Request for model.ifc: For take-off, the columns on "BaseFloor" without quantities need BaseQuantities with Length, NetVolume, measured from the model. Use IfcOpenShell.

First a look at what the model holds.

```python
import ifcopenshell
import ifcopenshell.util.element
import ifcopenshell.util.unit

model = ifcopenshell.open("model.ifc")
print(model.schema)
for unit_type in ("LENGTHUNIT", "AREAUNIT", "VOLUMEUNIT"):
    print(unit_type, ifcopenshell.util.unit.calculate_unit_scale(model, unit_type))
storey = next(s for s in model.by_type("IfcBuildingStorey") if s.Name == "BaseFloor")
columns = [e for e in ifcopenshell.util.element.get_decomposition(storey) if e.is_a("IfcColumn")]
for e in sorted(columns, key=lambda e: e.id()):
    print(e.id(), e.is_a(), e.Name, list(ifcopenshell.util.element.get_psets(e, qtos_only=True)), sep=" | ")
```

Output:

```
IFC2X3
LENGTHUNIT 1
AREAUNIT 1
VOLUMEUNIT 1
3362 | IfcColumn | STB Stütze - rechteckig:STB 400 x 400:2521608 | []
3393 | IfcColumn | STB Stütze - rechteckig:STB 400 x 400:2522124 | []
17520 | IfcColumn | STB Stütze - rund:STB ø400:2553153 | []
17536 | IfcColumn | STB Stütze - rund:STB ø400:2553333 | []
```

```python
import ifcopenshell
import ifcopenshell.api.pset
import ifcopenshell.geom
import ifcopenshell.util.element
import ifcopenshell.util.shape
import ifcopenshell.util.unit

model = ifcopenshell.open("model.ifc")
unit_scale = ifcopenshell.util.unit.calculate_unit_scale(model)
volume_scale = ifcopenshell.util.unit.calculate_unit_scale(model, "VOLUMEUNIT")
settings = ifcopenshell.geom.settings()

storey = next(s for s in model.by_type("IfcBuildingStorey") if s.Name == "BaseFloor")
columns = [e for e in ifcopenshell.util.element.get_decomposition(storey) if e.is_a("IfcColumn")]

for e in sorted(columns, key=lambda e: e.id()):
    if ifcopenshell.util.element.get_psets(e, qtos_only=True, should_inherit=False):
        continue
    # Geometry comes back in metres, in the element's own axes.
    shape = ifcopenshell.geom.create_shape(settings, e)
    values = {
        "Length": ifcopenshell.util.shape.get_z(shape.geometry) / unit_scale,
        "NetVolume": ifcopenshell.util.shape.get_volume(shape.geometry) / volume_scale,
    }
    qto = ifcopenshell.api.pset.add_qto(model, product=e, name="BaseQuantities")
    ifcopenshell.api.pset.edit_qto(model, qto=qto, properties=values)
    print(e.id(), {k: round(v, 3) for k, v in values.items()})

model.write("model_rev.ifc")
```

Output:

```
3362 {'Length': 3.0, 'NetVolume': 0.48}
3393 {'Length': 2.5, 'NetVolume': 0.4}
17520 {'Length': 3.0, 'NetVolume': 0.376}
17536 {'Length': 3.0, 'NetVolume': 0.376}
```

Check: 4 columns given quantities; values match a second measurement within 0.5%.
